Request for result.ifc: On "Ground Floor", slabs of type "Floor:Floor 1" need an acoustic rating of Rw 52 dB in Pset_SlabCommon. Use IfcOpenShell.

First a look at what the model holds.

```python
import ifcopenshell
import ifcopenshell.util.element

model = ifcopenshell.open("result.ifc")
print(model.schema)
storey = next(s for s in model.by_type("IfcBuildingStorey") if s.Name == "Ground Floor")
slabs = [e for e in ifcopenshell.util.element.get_decomposition(storey) if e.is_a("IfcSlab")]
seen = {}
for e in slabs:
    element_type = ifcopenshell.util.element.get_type(e)
    key = (element_type.Name if element_type != e and element_type else None, ifcopenshell.util.element.get_pset(e, "Pset_SlabCommon", "AcousticRating"))
    seen[key] = seen.get(key, 0) + 1
for (name, value), count in sorted(seen.items(), key=str):
    print(count, "x", name, "|", value)
```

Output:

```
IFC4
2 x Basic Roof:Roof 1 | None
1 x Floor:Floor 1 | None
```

```python
import ifcopenshell
import ifcopenshell.api.pset
import ifcopenshell.util.element

model = ifcopenshell.open("result.ifc")

storey = next(s for s in model.by_type("IfcBuildingStorey") if s.Name == "Ground Floor")
slabs = [e for e in ifcopenshell.util.element.get_decomposition(storey) if e.is_a("IfcSlab")]

count = 0
for e in slabs:
    element_type = ifcopenshell.util.element.get_type(e)
    if element_type in (None, e) or element_type.Name != "Floor:Floor 1":
        continue
    # add_pset returns the element's existing set when there is one.
    pset = ifcopenshell.api.pset.add_pset(model, product=e, name="Pset_SlabCommon")
    ifcopenshell.api.pset.edit_pset(model, pset=pset, properties={"AcousticRating": "Rw 52 dB"})
    count += 1

print(count, "slabs updated")

model.write("result_edited.ifc")
```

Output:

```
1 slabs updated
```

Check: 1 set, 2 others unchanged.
